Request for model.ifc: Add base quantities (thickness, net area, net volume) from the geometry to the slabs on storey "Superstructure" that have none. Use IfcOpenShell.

First a look at what the model holds.

```python
import ifcopenshell
import ifcopenshell.util.element
import ifcopenshell.util.unit

model = ifcopenshell.open("model.ifc")
print(model.schema)
for unit_type in ("LENGTHUNIT", "AREAUNIT", "VOLUMEUNIT"):
    print(unit_type, ifcopenshell.util.unit.calculate_unit_scale(model, unit_type))
storey = next(s for s in model.by_type("IfcBuildingStorey") if s.Name == "Superstructure")
slabs = [e for e in ifcopenshell.util.element.get_decomposition(storey) if e.is_a("IfcSlab")]
for e in sorted(slabs, key=lambda e: e.id()):
    print(e.id(), e.is_a(), e.Name, list(ifcopenshell.util.element.get_psets(e, qtos_only=True)), sep=" | ")
```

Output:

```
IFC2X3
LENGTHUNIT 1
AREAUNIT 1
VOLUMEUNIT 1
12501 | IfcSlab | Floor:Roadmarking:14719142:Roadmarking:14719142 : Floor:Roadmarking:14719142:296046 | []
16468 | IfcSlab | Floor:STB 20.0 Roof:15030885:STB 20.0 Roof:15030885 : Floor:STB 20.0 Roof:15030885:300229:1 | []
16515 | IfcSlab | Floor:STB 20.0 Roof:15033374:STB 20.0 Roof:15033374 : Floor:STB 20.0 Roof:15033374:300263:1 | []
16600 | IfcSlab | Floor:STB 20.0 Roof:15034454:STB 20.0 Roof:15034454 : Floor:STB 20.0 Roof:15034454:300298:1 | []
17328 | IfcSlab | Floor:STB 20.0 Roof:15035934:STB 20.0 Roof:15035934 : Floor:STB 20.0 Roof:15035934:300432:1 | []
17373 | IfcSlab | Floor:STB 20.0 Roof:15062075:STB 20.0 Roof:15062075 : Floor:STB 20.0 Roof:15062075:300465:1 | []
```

```python
import ifcopenshell
import ifcopenshell.api.pset
import ifcopenshell.geom
import ifcopenshell.util.element
import ifcopenshell.util.shape
import ifcopenshell.util.unit

model = ifcopenshell.open("model.ifc")
unit_scale = ifcopenshell.util.unit.calculate_unit_scale(model)
area_scale = ifcopenshell.util.unit.calculate_unit_scale(model, "AREAUNIT")
volume_scale = ifcopenshell.util.unit.calculate_unit_scale(model, "VOLUMEUNIT")
settings = ifcopenshell.geom.settings()

storey = next(s for s in model.by_type("IfcBuildingStorey") if s.Name == "Superstructure")
slabs = [e for e in ifcopenshell.util.element.get_decomposition(storey) if e.is_a("IfcSlab")]

for e in sorted(slabs, key=lambda e: e.id()):
    if ifcopenshell.util.element.get_psets(e, qtos_only=True, should_inherit=False):
        continue
    # Geometry comes back in metres, in the element's own axes.
    shape = ifcopenshell.geom.create_shape(settings, e)
    values = {
        "Width": ifcopenshell.util.shape.get_z(shape.geometry) / unit_scale,
        "NetArea": ifcopenshell.util.shape.get_footprint_area(shape.geometry) / area_scale,
        "NetVolume": ifcopenshell.util.shape.get_volume(shape.geometry) / volume_scale,
    }
    qto = ifcopenshell.api.pset.add_qto(model, product=e, name="BaseQuantities")
    ifcopenshell.api.pset.edit_qto(model, qto=qto, properties=values)
    print(e.id(), {k: round(v, 3) for k, v in values.items()})

model.write("model-out.ifc")
```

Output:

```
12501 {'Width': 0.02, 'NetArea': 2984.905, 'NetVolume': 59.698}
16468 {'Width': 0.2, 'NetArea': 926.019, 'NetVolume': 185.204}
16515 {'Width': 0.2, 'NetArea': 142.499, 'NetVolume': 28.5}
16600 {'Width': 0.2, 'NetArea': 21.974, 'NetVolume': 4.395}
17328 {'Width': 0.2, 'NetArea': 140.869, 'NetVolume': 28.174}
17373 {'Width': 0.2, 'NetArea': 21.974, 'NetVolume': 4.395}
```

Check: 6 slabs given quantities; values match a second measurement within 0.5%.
